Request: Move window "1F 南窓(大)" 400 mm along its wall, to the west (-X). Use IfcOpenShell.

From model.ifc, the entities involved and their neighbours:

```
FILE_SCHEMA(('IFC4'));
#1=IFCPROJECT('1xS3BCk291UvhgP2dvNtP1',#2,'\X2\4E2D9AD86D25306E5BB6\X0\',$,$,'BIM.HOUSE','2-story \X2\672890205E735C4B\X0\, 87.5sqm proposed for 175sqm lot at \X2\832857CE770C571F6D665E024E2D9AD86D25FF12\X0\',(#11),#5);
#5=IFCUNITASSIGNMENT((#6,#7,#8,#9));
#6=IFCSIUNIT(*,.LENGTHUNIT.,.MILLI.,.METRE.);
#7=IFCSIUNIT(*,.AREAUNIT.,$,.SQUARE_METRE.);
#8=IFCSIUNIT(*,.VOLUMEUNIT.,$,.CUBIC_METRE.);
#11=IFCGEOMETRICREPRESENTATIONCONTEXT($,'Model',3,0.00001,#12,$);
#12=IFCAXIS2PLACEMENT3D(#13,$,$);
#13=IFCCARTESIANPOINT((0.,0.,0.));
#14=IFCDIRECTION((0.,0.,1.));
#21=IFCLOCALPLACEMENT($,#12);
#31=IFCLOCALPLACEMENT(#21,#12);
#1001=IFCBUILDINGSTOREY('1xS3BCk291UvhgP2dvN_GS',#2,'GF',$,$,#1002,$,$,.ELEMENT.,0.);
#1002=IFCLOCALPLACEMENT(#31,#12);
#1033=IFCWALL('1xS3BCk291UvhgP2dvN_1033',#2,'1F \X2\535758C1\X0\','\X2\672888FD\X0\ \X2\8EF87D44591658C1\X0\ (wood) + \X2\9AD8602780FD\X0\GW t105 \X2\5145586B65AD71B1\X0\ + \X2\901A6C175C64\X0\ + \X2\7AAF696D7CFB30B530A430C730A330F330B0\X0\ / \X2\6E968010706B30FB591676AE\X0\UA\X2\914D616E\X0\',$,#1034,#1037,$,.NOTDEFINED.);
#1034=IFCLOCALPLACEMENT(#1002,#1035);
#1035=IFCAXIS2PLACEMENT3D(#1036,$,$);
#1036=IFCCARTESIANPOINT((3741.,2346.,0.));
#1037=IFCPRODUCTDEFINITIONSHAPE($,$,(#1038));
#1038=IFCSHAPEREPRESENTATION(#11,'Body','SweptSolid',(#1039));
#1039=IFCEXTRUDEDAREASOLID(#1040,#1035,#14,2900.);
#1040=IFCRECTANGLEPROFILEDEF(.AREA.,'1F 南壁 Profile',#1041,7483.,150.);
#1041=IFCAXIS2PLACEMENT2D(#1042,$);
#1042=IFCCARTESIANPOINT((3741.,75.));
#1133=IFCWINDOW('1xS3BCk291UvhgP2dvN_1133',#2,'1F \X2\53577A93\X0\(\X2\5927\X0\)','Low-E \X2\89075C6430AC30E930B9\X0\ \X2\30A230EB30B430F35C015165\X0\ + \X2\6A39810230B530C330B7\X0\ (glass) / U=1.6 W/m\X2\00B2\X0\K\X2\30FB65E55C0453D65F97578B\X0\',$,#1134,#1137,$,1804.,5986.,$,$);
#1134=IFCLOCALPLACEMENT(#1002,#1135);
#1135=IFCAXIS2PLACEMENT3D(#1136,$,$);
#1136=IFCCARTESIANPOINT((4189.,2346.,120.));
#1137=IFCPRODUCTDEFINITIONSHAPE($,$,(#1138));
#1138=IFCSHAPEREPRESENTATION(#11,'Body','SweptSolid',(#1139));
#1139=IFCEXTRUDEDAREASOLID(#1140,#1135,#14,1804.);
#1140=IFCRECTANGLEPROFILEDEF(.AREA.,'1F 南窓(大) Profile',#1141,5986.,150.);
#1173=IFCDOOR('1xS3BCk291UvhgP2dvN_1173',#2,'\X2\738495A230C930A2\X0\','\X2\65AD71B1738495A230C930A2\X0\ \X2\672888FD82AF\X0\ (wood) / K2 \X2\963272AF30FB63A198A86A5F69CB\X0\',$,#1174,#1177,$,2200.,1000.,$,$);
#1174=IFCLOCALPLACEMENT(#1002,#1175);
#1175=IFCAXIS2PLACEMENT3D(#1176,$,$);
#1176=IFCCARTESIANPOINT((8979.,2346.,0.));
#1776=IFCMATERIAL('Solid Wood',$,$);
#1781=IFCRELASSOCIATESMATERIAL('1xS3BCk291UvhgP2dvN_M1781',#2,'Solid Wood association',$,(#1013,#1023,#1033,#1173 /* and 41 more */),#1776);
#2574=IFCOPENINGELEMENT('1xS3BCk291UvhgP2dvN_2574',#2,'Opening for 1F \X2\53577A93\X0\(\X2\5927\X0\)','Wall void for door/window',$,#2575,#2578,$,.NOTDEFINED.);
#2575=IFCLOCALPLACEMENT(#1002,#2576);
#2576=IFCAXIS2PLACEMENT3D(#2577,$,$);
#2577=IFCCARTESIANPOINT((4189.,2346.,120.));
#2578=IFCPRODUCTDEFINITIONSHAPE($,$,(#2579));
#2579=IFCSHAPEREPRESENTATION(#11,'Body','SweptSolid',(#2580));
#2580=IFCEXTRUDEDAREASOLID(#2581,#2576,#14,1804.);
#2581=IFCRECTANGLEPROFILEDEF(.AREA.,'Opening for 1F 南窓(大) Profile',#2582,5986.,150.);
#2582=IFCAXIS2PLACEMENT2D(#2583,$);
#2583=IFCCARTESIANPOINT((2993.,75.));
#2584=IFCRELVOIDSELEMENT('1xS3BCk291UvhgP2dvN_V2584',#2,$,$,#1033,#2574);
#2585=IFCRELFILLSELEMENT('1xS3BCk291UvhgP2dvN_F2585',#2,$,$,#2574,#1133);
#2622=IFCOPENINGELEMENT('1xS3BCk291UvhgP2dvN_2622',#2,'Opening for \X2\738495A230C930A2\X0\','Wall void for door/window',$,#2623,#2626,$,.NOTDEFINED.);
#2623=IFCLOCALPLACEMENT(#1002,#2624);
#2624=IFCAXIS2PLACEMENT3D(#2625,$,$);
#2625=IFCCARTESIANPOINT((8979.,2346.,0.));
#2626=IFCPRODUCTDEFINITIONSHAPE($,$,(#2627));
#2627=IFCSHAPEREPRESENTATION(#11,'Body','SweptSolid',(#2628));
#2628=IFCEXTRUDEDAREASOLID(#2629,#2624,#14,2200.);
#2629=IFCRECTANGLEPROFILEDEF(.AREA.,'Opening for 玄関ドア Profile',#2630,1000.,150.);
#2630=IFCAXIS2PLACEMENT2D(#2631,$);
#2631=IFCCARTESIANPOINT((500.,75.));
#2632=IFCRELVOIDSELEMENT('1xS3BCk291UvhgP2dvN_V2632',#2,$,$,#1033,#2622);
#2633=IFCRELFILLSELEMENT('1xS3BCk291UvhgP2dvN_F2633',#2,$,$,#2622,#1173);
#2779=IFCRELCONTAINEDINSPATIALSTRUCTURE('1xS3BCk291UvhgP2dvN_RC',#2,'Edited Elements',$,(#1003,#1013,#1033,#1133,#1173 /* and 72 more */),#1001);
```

```python
import ifcopenshell
import ifcopenshell.api.geometry
import ifcopenshell.util.placement
import ifcopenshell.util.unit

model = ifcopenshell.open("model.ifc")
unit_scale = ifcopenshell.util.unit.calculate_unit_scale(model)

window = model.by_guid("1xS3BCk291UvhgP2dvN_1133")
opening = window.FillsVoids[0].RelatingOpeningElement
wall = opening.VoidsElements[0].RelatingBuildingElement

wall_matrix = ifcopenshell.util.placement.get_local_placement(wall.ObjectPlacement)
shift = wall_matrix[:3, 0] * -0.4 / unit_scale
before = ifcopenshell.util.placement.get_local_placement(window.ObjectPlacement)[:3, 3].copy()

# The window is not placed relative to its opening, so move both.
for product in (opening, window):
    matrix = ifcopenshell.util.placement.get_local_placement(product.ObjectPlacement)
    matrix[:3, 3] += shift
    ifcopenshell.api.geometry.edit_object_placement(model, product=product, matrix=matrix, is_si=False)

after = ifcopenshell.util.placement.get_local_placement(window.ObjectPlacement)[:3, 3]
print("window moved by", (after - before).round(3) + 0.0)

model.write("model_updated.ifc")
```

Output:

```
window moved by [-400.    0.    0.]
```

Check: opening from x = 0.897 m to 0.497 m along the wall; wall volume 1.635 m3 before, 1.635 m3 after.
